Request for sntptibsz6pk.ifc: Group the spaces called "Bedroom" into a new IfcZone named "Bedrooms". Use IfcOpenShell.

First a look at what the model holds.

```python
import ifcopenshell

model = ifcopenshell.open("sntptibsz6pk.ifc")
print(model.schema)
seen = {}
for space in model.by_type("IfcSpace"):
    seen[space.Name] = seen.get(space.Name, 0) + 1
for name, count in sorted(seen.items(), key=str):
    print(count, "x", name)
print("zones:", [z.Name for z in model.by_type("IfcZone")][:20])
```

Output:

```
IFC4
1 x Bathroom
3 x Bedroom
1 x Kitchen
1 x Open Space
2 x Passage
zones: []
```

```python
import ifcopenshell
import ifcopenshell.api.group
import ifcopenshell.api.root

model = ifcopenshell.open("sntptibsz6pk.ifc")

names = {"Bedroom"}
spaces = [s for s in model.by_type("IfcSpace") if s.Name in names]

zone = ifcopenshell.api.root.create_entity(model, ifc_class="IfcZone", name="Bedrooms")
ifcopenshell.api.group.assign_group(model, products=spaces, group=zone)
print(len(spaces), "spaces in", zone.Name)

model.write("sntptibsz6pk_edited.ifc")
```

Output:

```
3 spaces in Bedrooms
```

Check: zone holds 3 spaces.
